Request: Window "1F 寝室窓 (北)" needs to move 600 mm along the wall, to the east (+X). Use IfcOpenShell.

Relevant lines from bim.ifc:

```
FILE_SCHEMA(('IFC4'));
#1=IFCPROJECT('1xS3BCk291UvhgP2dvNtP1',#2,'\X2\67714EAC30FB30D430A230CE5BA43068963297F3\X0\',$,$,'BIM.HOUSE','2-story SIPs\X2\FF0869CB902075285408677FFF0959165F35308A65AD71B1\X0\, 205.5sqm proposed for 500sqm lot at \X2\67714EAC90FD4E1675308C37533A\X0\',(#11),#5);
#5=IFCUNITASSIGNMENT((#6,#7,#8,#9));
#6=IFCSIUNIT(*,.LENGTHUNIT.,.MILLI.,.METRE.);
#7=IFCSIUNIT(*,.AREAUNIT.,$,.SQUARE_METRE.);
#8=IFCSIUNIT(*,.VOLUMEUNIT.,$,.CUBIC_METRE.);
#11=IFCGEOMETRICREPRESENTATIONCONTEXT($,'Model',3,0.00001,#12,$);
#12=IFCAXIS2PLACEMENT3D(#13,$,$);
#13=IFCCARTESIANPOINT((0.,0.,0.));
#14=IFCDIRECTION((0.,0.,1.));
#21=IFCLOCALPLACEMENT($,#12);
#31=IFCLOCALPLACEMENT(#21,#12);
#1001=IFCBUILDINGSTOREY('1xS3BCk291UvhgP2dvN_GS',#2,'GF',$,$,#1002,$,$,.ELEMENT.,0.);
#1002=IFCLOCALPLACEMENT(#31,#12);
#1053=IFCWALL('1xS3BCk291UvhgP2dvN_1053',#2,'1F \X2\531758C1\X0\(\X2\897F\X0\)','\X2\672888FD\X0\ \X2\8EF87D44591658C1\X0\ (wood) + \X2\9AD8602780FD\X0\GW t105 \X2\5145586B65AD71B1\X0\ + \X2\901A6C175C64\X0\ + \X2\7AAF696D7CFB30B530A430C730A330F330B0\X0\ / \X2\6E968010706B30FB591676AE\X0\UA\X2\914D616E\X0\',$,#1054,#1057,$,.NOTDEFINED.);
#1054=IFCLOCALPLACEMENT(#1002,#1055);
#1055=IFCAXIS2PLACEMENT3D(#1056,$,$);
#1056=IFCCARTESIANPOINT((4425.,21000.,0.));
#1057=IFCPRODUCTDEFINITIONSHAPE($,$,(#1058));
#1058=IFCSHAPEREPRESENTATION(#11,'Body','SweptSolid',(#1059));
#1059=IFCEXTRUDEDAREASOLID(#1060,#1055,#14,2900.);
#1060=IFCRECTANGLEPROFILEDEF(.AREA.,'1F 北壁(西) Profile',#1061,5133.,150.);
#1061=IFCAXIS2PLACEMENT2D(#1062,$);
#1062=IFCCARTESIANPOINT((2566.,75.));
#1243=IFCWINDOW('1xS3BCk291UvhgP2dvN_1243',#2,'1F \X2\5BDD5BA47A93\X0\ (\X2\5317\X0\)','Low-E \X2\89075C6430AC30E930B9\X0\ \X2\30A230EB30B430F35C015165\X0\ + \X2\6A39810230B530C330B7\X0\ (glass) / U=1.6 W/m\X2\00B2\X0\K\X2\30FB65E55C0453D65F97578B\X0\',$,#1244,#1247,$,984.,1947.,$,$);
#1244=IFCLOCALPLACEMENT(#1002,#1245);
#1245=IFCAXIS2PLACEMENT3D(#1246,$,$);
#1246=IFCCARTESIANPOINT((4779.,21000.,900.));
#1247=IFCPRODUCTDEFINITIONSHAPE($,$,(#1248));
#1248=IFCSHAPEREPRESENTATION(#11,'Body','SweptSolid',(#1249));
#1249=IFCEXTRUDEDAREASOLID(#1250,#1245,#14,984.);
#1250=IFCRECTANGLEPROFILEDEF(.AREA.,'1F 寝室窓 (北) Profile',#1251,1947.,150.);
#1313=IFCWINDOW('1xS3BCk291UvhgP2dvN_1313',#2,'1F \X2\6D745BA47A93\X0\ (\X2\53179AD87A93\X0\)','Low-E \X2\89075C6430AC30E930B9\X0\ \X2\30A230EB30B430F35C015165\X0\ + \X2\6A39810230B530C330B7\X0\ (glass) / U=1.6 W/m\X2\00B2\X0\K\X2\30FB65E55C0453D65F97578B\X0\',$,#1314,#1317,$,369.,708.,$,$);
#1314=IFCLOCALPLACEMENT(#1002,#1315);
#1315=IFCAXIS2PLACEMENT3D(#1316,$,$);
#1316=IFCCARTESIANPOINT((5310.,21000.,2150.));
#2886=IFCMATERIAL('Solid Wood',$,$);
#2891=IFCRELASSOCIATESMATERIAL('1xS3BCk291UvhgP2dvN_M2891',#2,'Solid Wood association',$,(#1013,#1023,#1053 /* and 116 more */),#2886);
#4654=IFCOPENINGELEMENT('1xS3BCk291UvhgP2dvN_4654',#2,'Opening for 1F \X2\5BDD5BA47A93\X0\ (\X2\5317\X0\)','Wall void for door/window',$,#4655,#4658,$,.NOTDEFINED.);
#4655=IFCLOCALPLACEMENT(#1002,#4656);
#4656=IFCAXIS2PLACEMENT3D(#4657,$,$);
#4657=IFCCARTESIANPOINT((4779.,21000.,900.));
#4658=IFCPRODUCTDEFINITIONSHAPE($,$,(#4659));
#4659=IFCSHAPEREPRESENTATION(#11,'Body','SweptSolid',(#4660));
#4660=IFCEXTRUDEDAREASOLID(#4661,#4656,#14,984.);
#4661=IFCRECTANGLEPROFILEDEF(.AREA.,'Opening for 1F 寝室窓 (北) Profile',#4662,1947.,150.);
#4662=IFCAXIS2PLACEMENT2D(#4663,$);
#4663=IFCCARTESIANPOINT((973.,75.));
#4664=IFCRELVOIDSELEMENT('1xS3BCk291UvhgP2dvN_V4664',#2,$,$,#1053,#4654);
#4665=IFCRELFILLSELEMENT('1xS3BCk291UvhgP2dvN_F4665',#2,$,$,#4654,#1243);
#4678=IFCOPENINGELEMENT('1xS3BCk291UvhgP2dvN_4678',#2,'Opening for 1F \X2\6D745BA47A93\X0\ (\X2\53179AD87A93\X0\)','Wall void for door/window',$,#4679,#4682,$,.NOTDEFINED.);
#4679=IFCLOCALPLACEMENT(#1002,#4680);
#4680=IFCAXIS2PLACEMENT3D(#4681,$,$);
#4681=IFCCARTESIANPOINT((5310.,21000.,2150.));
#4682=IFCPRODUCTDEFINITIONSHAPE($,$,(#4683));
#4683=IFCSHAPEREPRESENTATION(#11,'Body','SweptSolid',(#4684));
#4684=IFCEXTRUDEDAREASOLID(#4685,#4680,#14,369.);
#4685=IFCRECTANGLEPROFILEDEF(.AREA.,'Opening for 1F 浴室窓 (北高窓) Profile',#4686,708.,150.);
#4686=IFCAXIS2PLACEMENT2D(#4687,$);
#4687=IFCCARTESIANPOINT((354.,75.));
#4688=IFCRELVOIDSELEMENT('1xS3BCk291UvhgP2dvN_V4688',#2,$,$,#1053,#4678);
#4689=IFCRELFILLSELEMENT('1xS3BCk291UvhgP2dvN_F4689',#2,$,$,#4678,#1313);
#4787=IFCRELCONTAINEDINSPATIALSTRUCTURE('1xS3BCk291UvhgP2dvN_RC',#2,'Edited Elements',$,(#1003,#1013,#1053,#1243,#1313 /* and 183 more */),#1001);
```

```python
import ifcopenshell
import ifcopenshell.api.geometry
import ifcopenshell.util.placement
import ifcopenshell.util.unit

model = ifcopenshell.open("bim.ifc")
unit_scale = ifcopenshell.util.unit.calculate_unit_scale(model)

window = model.by_guid("1xS3BCk291UvhgP2dvN_1243")
opening = window.FillsVoids[0].RelatingOpeningElement
wall = opening.VoidsElements[0].RelatingBuildingElement

wall_matrix = ifcopenshell.util.placement.get_local_placement(wall.ObjectPlacement)
shift = wall_matrix[:3, 0] * 0.6 / unit_scale
before = ifcopenshell.util.placement.get_local_placement(window.ObjectPlacement)[:3, 3].copy()

# The window is not placed relative to its opening, so move both.
for product in (opening, window):
    matrix = ifcopenshell.util.placement.get_local_placement(product.ObjectPlacement)
    matrix[:3, 3] += shift
    ifcopenshell.api.geometry.edit_object_placement(model, product=product, matrix=matrix, is_si=False)

after = ifcopenshell.util.placement.get_local_placement(window.ObjectPlacement)[:3, 3]
print("window moved by", (after - before).round(3) + 0.0)

model.write("bim_edited.ifc")
```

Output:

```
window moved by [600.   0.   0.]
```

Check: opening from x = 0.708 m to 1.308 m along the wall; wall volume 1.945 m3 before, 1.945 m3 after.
